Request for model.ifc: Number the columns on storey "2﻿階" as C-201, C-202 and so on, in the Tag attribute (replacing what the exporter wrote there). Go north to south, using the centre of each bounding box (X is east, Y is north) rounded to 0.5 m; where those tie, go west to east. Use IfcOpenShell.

First a look at what the model holds.

```python
import ifcopenshell
import ifcopenshell.util.element
import ifcopenshell.util.placement

model = ifcopenshell.open("model.ifc")
print(model.schema)
storey = next(s for s in model.by_type("IfcBuildingStorey") if s.Name == '2\ufeff階')
columns = [e for e in ifcopenshell.util.element.get_decomposition(storey) if e.is_a("IfcColumn")]
for e in sorted(columns, key=lambda e: e.id()):
    origin = ifcopenshell.util.placement.get_local_placement(e.ObjectPlacement)[:3, 3]
    print(e.id(), e.Tag, e.Name, origin.round(2) + 0.0, sep=" | ")
```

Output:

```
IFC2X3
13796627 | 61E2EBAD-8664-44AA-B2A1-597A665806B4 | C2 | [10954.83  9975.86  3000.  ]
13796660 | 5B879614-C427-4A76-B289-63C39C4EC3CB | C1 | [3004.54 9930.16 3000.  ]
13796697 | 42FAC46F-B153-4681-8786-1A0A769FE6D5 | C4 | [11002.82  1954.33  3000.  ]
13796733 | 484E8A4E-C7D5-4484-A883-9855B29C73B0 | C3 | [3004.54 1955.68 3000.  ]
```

```python
import ifcopenshell
import ifcopenshell.geom
import ifcopenshell.util.element
import ifcopenshell.util.shape

model = ifcopenshell.open("model.ifc")
settings = ifcopenshell.geom.settings()
settings.set("use-world-coords", True)


def centre(element):
    shape = ifcopenshell.geom.create_shape(settings, element)
    return ifcopenshell.util.shape.get_bbox_centroid(shape.geometry)


storey = next(s for s in model.by_type("IfcBuildingStorey") if s.Name == '2\ufeff階')
columns = [e for e in ifcopenshell.util.element.get_decomposition(storey) if e.is_a("IfcColumn")]

# Insertion points can sit at a corner or the storey origin, so sort by the geometry (in metres).
centres = {e: centre(e) for e in columns}
columns.sort(key=lambda e: (-round(centres[e][1] / 0.5), centres[e][0]))

for i, e in enumerate(columns, start=1):
    number = f"C-2{i:02d}"
    e.Tag = number
    print(e.id(), number)

model.write("model_edited.ifc")
```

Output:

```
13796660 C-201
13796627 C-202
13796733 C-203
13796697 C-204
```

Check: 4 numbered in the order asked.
